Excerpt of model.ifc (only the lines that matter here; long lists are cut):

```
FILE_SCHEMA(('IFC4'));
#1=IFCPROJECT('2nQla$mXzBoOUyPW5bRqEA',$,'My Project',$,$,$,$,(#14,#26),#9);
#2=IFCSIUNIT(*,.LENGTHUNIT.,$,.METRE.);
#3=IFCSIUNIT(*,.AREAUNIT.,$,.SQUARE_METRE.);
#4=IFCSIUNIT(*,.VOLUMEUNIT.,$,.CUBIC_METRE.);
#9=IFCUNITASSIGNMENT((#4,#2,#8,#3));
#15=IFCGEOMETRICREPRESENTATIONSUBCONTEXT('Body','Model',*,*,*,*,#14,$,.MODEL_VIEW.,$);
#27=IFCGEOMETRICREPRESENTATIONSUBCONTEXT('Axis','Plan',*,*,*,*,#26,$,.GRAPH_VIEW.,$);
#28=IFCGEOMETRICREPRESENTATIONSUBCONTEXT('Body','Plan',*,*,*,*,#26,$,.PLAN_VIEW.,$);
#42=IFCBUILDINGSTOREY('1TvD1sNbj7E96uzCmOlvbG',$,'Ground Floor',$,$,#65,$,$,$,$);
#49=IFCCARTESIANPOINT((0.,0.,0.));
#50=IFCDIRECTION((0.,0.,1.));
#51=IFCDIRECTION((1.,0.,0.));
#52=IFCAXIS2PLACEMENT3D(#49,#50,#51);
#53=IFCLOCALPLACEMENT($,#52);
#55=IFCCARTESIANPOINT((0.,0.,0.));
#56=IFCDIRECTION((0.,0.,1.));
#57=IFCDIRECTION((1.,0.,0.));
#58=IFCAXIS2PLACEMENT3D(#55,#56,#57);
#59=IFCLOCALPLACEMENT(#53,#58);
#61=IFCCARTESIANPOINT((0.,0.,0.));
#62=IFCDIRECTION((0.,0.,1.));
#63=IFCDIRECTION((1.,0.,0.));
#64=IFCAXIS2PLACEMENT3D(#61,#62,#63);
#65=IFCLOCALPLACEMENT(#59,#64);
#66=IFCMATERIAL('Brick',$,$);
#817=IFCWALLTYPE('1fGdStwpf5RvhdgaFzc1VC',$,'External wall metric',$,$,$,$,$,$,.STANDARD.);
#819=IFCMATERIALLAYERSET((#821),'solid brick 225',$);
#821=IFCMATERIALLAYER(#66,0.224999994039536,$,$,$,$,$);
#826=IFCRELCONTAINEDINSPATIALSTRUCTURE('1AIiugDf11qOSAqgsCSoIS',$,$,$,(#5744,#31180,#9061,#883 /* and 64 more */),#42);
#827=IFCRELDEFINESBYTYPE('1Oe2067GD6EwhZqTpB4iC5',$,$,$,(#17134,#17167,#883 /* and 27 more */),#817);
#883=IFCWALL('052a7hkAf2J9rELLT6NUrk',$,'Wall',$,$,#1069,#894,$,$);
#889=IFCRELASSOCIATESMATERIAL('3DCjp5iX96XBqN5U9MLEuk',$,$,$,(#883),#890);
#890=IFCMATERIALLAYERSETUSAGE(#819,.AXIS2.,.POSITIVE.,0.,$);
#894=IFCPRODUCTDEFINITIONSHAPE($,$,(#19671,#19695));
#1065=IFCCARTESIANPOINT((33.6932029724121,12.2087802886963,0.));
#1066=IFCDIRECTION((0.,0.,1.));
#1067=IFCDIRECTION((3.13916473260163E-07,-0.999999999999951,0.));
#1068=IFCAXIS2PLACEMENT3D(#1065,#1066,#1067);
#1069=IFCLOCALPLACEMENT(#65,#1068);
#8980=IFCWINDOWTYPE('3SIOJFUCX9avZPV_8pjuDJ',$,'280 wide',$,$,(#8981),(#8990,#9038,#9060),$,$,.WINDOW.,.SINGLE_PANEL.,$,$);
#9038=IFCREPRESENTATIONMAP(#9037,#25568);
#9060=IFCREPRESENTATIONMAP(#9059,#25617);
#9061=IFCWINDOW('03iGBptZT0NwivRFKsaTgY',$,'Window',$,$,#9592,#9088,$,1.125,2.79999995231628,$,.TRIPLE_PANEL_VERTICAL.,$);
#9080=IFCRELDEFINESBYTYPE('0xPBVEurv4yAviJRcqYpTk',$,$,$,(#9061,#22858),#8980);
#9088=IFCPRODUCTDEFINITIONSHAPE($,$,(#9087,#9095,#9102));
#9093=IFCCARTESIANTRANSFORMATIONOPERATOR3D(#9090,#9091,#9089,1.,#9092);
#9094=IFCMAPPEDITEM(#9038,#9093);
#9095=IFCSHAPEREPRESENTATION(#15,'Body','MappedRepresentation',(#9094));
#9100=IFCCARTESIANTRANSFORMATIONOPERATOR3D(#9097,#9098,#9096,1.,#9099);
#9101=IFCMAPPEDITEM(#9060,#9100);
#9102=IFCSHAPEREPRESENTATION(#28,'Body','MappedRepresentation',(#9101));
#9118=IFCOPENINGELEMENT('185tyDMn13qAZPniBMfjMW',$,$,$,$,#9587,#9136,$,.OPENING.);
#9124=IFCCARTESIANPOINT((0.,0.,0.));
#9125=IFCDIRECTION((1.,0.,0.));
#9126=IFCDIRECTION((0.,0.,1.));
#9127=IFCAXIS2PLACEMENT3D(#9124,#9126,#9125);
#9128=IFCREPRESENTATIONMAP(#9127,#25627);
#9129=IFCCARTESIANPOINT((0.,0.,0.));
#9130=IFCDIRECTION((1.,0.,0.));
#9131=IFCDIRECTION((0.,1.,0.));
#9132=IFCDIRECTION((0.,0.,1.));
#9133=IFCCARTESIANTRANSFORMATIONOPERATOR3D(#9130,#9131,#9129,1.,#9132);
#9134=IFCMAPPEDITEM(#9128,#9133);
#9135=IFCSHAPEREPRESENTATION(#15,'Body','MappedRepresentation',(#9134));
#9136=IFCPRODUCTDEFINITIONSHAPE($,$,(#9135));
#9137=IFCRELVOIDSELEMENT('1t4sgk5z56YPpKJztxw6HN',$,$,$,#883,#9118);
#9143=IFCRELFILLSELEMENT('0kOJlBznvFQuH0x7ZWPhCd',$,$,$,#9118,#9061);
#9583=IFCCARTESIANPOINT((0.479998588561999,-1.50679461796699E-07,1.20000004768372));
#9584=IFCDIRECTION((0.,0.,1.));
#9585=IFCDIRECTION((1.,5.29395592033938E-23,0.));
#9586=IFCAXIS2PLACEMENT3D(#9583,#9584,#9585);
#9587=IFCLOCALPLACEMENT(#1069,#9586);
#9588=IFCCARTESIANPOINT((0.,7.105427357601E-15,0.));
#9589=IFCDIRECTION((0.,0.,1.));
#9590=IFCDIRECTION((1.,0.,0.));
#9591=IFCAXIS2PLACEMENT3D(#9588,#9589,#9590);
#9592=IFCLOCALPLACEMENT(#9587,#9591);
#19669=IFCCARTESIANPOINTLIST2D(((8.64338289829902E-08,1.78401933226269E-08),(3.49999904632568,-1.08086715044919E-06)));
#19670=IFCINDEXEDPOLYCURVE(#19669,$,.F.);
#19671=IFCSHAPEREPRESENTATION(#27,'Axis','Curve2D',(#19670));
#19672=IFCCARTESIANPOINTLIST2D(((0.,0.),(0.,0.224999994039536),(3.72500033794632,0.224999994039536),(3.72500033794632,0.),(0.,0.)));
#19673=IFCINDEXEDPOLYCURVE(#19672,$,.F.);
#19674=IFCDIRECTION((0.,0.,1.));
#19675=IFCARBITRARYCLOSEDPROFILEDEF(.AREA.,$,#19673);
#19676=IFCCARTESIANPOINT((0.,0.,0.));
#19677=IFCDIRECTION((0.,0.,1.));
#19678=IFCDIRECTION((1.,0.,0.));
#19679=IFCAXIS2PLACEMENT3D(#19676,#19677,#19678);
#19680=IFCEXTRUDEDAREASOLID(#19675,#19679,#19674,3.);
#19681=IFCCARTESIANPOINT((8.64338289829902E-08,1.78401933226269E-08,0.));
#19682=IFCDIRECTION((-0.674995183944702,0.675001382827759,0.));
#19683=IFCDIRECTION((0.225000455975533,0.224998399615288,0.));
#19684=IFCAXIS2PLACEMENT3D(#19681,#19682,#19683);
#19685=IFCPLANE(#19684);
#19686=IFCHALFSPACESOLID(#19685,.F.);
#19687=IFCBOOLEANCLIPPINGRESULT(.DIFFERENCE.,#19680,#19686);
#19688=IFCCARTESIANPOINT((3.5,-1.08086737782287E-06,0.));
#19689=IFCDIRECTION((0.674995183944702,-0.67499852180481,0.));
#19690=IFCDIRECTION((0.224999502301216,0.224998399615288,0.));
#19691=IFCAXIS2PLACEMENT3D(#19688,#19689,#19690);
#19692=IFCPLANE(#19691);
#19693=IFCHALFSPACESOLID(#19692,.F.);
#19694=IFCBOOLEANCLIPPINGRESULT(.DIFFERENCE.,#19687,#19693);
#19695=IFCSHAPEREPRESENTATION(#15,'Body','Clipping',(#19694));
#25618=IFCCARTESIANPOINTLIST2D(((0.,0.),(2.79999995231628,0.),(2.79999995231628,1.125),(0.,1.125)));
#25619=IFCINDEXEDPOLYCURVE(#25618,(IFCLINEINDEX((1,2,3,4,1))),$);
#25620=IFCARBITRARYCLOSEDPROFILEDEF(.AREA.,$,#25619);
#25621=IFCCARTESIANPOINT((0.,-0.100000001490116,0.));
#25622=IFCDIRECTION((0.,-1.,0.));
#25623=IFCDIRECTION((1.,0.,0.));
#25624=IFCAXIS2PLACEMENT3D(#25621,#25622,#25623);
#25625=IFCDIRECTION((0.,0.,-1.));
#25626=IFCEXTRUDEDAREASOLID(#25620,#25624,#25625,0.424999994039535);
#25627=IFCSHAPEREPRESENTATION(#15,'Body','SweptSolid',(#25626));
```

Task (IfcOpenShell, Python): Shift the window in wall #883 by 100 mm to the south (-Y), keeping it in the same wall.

```python
import ifcopenshell
import ifcopenshell.api.geometry
import ifcopenshell.util.placement
import ifcopenshell.util.unit

model = ifcopenshell.open("model.ifc")
unit_scale = ifcopenshell.util.unit.calculate_unit_scale(model)

window = model.by_id(9061)
opening = window.FillsVoids[0].RelatingOpeningElement
wall = opening.VoidsElements[0].RelatingBuildingElement

wall_matrix = ifcopenshell.util.placement.get_local_placement(wall.ObjectPlacement)
shift = wall_matrix[:3, 0] * 0.1 / unit_scale
before = ifcopenshell.util.placement.get_local_placement(window.ObjectPlacement)[:3, 3].copy()

# The window is placed relative to its opening, so it follows when the opening moves.
matrix = ifcopenshell.util.placement.get_local_placement(opening.ObjectPlacement)
matrix[:3, 3] += shift
ifcopenshell.api.geometry.edit_object_placement(
    model, product=opening, matrix=matrix, is_si=False, should_transform_children=True
)

after = ifcopenshell.util.placement.get_local_placement(window.ObjectPlacement)[:3, 3]
print("window moved by", (after - before).round(3) + 0.0)

model.write("model_updated.ifc")
```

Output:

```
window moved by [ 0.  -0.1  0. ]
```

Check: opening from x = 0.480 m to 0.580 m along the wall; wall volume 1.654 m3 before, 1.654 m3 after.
